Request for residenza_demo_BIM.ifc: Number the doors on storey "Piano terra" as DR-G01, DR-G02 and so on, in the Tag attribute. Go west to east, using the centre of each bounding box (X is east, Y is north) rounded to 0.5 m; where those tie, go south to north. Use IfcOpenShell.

First a look at what the model holds.

```python
import ifcopenshell
import ifcopenshell.util.element
import ifcopenshell.util.placement

model = ifcopenshell.open("residenza_demo_BIM.ifc")
print(model.schema)
storey = next(s for s in model.by_type("IfcBuildingStorey") if s.Name == "Piano terra")
doors = [e for e in ifcopenshell.util.element.get_decomposition(storey) if e.is_a("IfcDoor")]
for e in sorted(doors, key=lambda e: e.id()):
    origin = ifcopenshell.util.placement.get_local_placement(e.ObjectPlacement)[:3, 3]
    print(e.id(), e.Tag, e.Name, origin.round(2) + 0.0, sep=" | ")
```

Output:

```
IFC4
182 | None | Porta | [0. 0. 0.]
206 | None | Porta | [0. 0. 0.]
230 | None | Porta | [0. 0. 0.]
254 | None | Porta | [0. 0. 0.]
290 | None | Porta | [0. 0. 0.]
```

```python
import ifcopenshell
import ifcopenshell.geom
import ifcopenshell.util.element
import ifcopenshell.util.shape

model = ifcopenshell.open("residenza_demo_BIM.ifc")
settings = ifcopenshell.geom.settings()
settings.set("use-world-coords", True)


def centre(element):
    shape = ifcopenshell.geom.create_shape(settings, element)
    return ifcopenshell.util.shape.get_bbox_centroid(shape.geometry)


storey = next(s for s in model.by_type("IfcBuildingStorey") if s.Name == "Piano terra")
doors = [e for e in ifcopenshell.util.element.get_decomposition(storey) if e.is_a("IfcDoor")]

# Insertion points can sit at a corner or the storey origin, so sort by the geometry (in metres).
centres = {e: centre(e) for e in doors}
doors.sort(key=lambda e: (round(centres[e][0] / 0.5), centres[e][1]))

for i, e in enumerate(doors, start=1):
    number = f"DR-G{i:02d}"
    e.Tag = number
    print(e.id(), number)

model.write("residenza_demo_BIM_updated.ifc")
```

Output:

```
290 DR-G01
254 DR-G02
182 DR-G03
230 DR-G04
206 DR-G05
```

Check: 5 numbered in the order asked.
